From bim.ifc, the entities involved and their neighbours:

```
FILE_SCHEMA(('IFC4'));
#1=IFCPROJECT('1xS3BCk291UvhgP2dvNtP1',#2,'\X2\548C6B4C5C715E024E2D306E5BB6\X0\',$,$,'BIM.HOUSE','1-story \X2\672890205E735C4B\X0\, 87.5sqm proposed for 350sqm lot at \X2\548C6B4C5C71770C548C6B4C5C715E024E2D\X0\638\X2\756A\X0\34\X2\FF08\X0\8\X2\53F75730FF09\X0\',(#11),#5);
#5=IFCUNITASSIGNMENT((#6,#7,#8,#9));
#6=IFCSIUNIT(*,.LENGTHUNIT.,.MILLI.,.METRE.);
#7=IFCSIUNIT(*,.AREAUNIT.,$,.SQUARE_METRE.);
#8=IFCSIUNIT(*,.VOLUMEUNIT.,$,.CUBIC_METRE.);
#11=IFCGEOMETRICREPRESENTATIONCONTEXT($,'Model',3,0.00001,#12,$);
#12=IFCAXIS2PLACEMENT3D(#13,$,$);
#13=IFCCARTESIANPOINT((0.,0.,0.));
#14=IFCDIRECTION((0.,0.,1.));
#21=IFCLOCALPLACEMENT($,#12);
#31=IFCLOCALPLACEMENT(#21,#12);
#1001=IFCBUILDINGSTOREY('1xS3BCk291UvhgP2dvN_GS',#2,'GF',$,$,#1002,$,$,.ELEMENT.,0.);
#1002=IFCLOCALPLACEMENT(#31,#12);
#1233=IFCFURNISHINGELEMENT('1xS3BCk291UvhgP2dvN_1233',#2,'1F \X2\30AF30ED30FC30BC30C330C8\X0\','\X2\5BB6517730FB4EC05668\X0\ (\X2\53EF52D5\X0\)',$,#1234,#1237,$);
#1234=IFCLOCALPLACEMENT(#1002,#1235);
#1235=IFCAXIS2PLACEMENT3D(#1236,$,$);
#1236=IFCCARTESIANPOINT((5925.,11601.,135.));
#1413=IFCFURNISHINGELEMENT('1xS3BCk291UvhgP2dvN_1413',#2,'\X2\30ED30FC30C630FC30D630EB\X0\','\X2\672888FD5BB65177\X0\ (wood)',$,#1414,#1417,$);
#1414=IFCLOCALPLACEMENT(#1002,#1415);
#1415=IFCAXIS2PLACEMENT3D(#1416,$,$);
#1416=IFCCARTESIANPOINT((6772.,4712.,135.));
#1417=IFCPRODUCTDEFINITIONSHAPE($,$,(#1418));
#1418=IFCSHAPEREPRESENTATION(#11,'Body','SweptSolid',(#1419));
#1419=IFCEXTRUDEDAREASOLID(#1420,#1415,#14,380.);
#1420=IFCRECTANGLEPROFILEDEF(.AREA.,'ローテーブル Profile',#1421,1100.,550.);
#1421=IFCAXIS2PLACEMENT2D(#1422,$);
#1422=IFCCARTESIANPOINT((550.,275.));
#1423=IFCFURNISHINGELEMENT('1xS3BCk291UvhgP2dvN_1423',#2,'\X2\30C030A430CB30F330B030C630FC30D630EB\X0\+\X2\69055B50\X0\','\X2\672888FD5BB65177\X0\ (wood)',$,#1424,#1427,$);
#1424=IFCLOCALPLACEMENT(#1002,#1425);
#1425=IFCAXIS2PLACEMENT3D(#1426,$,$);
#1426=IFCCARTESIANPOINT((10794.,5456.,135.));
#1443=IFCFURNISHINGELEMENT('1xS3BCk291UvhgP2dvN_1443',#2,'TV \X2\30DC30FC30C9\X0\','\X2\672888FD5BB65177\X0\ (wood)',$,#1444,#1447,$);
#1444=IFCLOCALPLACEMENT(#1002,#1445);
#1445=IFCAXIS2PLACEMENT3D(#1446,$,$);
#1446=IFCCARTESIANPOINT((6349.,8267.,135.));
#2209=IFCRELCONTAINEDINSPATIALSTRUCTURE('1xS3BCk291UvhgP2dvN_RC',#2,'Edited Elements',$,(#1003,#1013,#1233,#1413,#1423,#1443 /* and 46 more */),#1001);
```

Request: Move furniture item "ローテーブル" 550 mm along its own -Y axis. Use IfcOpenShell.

```python
import ifcopenshell
import ifcopenshell.api.geometry
import ifcopenshell.util.placement
import ifcopenshell.util.unit

model = ifcopenshell.open("bim.ifc")
unit_scale = ifcopenshell.util.unit.calculate_unit_scale(model)

item = model.by_guid("1xS3BCk291UvhgP2dvN_1413")
matrix = ifcopenshell.util.placement.get_local_placement(item.ObjectPlacement)
matrix[:3, 3] -= matrix[:3, 1] * 0.55 / unit_scale
ifcopenshell.api.geometry.edit_object_placement(model, product=item, matrix=matrix, is_si=False)

print(ifcopenshell.util.placement.get_local_placement(item.ObjectPlacement).round(3) + 0.0)

model.write("bim_v2.ifc")
```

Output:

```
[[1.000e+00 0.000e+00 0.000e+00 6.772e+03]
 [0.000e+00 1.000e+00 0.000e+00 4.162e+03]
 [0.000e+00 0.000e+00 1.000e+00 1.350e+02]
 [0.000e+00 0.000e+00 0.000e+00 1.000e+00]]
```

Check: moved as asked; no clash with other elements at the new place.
